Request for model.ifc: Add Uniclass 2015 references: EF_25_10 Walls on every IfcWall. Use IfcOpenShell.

First a look at what the model holds.

```python
import ifcopenshell

model = ifcopenshell.open("model.ifc")
print(model.schema)
print("classifications:", [c.Name for c in model.by_type("IfcClassification")])
for ifc_class in ("IfcDoor", "IfcRoof", "IfcStair", "IfcWall", "IfcWindow"):
    print(ifc_class, len(model.by_type(ifc_class)))
```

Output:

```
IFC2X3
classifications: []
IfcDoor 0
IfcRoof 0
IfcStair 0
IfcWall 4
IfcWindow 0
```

```python
import ifcopenshell
import ifcopenshell.api.classification

model = ifcopenshell.open("model.ifc")

# IFC2X3 requires Source and Edition and has no link from the project to the system.
system = model.create_entity("IfcClassification", Source="NBS", Edition="2015", Name="Uniclass 2015")

codes = {
    "IfcWall": ("EF_25_10", "Walls"),
}
for ifc_class, (code, name) in codes.items():
    products = model.by_type(ifc_class)
    ifcopenshell.api.classification.add_reference(
        model, products=products, classification=system, identification=code, name=name
    )
    print(code, len(products))

model.write("model_v2.ifc")
```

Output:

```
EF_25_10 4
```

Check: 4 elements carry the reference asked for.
